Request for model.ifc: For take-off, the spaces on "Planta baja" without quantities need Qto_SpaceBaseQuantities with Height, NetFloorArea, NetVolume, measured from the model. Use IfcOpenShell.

First a look at what the model holds.

```python
import ifcopenshell
import ifcopenshell.util.element
import ifcopenshell.util.unit

model = ifcopenshell.open("model.ifc")
print(model.schema)
for unit_type in ("LENGTHUNIT", "AREAUNIT", "VOLUMEUNIT"):
    print(unit_type, ifcopenshell.util.unit.calculate_unit_scale(model, unit_type))
storey = next(s for s in model.by_type("IfcBuildingStorey") if s.Name == "Planta baja")
spaces = [e for e in ifcopenshell.util.element.get_decomposition(storey) if e.is_a("IfcSpace")]
for e in sorted(spaces, key=lambda e: e.id()):
    print(e.id(), e.is_a(), e.Name, list(ifcopenshell.util.element.get_psets(e, qtos_only=True)), sep=" | ")
```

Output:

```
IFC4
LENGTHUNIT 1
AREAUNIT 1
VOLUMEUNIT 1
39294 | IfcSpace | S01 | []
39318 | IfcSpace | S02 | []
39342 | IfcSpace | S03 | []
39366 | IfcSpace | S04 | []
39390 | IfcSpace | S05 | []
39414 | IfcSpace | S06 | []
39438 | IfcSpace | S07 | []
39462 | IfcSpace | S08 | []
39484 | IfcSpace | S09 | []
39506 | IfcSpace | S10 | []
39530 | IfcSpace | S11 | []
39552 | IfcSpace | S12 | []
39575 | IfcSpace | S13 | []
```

```python
import ifcopenshell
import ifcopenshell.api.pset
import ifcopenshell.geom
import ifcopenshell.util.element
import ifcopenshell.util.shape
import ifcopenshell.util.unit

model = ifcopenshell.open("model.ifc")
unit_scale = ifcopenshell.util.unit.calculate_unit_scale(model)
area_scale = ifcopenshell.util.unit.calculate_unit_scale(model, "AREAUNIT")
volume_scale = ifcopenshell.util.unit.calculate_unit_scale(model, "VOLUMEUNIT")
settings = ifcopenshell.geom.settings()

storey = next(s for s in model.by_type("IfcBuildingStorey") if s.Name == "Planta baja")
spaces = [e for e in ifcopenshell.util.element.get_decomposition(storey) if e.is_a("IfcSpace")]

for e in sorted(spaces, key=lambda e: e.id()):
    if ifcopenshell.util.element.get_psets(e, qtos_only=True, should_inherit=False):
        continue
    # Geometry comes back in metres, in the element's own axes.
    shape = ifcopenshell.geom.create_shape(settings, e)
    values = {
        "Height": ifcopenshell.util.shape.get_z(shape.geometry) / unit_scale,
        "NetFloorArea": ifcopenshell.util.shape.get_footprint_area(shape.geometry) / area_scale,
        "NetVolume": ifcopenshell.util.shape.get_volume(shape.geometry) / volume_scale,
    }
    qto = ifcopenshell.api.pset.add_qto(model, product=e, name="Qto_SpaceBaseQuantities")
    ifcopenshell.api.pset.edit_qto(model, qto=qto, properties=values)
    print(e.id(), {k: round(v, 3) for k, v in values.items()})

model.write("model_v2.ifc")
```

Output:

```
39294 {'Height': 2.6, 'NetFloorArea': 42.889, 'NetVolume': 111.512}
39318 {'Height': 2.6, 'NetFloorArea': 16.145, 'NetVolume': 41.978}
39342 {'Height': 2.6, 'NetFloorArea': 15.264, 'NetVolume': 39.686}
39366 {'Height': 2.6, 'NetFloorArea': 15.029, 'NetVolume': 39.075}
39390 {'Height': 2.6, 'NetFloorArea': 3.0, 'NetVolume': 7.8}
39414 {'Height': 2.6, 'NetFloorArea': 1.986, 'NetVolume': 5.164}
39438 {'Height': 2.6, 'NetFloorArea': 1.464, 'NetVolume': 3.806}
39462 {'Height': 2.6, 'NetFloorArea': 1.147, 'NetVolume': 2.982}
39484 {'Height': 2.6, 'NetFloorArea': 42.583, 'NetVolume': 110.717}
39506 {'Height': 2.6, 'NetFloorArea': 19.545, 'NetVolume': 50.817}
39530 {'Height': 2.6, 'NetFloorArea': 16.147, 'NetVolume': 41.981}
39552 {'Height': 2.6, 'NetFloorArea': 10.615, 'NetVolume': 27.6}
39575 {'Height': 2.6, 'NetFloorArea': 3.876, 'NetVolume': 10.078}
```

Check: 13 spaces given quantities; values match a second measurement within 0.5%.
